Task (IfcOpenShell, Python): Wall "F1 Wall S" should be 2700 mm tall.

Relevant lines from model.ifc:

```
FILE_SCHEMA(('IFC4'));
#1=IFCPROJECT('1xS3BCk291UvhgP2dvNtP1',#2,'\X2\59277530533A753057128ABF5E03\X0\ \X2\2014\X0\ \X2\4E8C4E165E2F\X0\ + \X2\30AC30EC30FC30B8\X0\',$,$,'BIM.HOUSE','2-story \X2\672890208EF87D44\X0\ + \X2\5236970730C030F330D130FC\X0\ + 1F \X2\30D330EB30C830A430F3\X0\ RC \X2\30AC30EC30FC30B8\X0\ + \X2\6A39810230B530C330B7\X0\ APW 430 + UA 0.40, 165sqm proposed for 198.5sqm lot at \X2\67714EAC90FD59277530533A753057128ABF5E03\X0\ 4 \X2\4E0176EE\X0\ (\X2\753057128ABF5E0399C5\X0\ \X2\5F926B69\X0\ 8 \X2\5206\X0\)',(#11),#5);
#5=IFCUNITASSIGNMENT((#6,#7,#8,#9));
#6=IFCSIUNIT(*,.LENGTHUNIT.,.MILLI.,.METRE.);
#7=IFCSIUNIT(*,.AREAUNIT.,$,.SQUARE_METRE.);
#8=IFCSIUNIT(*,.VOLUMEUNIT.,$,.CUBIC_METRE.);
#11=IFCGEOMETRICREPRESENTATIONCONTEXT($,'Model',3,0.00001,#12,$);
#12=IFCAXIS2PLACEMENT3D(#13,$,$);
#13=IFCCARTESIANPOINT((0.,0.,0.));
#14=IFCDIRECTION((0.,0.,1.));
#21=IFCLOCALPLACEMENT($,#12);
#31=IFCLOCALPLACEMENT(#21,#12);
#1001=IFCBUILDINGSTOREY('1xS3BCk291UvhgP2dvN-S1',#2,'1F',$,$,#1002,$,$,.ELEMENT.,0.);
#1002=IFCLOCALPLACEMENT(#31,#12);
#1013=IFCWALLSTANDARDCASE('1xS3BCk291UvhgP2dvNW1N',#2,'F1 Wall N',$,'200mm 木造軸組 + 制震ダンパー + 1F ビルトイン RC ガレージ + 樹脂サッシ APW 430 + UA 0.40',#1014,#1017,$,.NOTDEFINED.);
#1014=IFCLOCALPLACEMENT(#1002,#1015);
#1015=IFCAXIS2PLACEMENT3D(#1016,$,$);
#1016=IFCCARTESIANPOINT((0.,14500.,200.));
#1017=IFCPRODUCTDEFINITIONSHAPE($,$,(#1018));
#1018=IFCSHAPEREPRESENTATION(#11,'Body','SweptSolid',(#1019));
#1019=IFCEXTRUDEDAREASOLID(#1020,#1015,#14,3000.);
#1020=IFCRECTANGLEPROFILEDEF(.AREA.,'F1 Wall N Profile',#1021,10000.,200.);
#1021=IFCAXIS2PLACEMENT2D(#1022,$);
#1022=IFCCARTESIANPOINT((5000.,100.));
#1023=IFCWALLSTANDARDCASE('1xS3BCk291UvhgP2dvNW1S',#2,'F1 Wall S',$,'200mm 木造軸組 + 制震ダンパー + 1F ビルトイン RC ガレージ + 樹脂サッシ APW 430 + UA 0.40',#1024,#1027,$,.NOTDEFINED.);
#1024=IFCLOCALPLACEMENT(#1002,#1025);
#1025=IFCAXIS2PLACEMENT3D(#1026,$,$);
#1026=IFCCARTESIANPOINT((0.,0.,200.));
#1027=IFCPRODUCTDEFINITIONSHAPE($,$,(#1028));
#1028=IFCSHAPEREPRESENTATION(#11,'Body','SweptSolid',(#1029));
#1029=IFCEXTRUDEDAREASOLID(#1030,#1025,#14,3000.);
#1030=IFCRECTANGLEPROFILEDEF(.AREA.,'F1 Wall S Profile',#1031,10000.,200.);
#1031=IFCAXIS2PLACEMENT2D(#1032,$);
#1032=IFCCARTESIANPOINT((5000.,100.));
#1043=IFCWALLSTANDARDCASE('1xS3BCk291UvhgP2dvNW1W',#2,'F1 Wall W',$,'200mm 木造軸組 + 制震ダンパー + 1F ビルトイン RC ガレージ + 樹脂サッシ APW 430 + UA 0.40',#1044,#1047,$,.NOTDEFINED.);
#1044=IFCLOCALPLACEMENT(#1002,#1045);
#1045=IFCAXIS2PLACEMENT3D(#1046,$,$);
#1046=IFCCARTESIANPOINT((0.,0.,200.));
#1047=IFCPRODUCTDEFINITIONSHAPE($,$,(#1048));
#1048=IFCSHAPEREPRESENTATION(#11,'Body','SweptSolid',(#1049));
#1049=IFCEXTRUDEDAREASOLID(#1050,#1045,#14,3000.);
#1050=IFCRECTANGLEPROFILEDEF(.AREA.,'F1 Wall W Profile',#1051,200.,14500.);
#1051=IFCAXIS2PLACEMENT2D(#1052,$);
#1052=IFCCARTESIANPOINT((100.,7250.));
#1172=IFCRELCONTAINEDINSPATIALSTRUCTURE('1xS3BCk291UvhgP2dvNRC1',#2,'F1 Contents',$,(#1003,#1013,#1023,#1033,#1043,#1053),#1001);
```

```python
import ifcopenshell
import ifcopenshell.geom
import ifcopenshell.util.shape
import ifcopenshell.util.unit

model = ifcopenshell.open("model.ifc")
unit_scale = ifcopenshell.util.unit.calculate_unit_scale(model)
settings = ifcopenshell.geom.settings()


def volume(element):
    """Net volume in cubic metres, openings subtracted."""
    shape = ifcopenshell.geom.create_shape(settings, element)
    return ifcopenshell.util.shape.get_volume(shape.geometry)


wall = model.by_id(1023)
before = volume(wall)

body = next(r for r in wall.Representation.Representations if r.RepresentationIdentifier == "Body")
solid = body.Items[0]
old_height = solid.Depth
solid.Depth = 2.7 / unit_scale
after = volume(wall)

print(f"height {old_height:g} -> {solid.Depth:g}, volume {before:.3f} -> {after:.3f} m3")

model.write("model_edited.ifc")
```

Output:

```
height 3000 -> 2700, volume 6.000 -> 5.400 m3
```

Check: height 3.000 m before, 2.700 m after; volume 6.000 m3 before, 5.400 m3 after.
